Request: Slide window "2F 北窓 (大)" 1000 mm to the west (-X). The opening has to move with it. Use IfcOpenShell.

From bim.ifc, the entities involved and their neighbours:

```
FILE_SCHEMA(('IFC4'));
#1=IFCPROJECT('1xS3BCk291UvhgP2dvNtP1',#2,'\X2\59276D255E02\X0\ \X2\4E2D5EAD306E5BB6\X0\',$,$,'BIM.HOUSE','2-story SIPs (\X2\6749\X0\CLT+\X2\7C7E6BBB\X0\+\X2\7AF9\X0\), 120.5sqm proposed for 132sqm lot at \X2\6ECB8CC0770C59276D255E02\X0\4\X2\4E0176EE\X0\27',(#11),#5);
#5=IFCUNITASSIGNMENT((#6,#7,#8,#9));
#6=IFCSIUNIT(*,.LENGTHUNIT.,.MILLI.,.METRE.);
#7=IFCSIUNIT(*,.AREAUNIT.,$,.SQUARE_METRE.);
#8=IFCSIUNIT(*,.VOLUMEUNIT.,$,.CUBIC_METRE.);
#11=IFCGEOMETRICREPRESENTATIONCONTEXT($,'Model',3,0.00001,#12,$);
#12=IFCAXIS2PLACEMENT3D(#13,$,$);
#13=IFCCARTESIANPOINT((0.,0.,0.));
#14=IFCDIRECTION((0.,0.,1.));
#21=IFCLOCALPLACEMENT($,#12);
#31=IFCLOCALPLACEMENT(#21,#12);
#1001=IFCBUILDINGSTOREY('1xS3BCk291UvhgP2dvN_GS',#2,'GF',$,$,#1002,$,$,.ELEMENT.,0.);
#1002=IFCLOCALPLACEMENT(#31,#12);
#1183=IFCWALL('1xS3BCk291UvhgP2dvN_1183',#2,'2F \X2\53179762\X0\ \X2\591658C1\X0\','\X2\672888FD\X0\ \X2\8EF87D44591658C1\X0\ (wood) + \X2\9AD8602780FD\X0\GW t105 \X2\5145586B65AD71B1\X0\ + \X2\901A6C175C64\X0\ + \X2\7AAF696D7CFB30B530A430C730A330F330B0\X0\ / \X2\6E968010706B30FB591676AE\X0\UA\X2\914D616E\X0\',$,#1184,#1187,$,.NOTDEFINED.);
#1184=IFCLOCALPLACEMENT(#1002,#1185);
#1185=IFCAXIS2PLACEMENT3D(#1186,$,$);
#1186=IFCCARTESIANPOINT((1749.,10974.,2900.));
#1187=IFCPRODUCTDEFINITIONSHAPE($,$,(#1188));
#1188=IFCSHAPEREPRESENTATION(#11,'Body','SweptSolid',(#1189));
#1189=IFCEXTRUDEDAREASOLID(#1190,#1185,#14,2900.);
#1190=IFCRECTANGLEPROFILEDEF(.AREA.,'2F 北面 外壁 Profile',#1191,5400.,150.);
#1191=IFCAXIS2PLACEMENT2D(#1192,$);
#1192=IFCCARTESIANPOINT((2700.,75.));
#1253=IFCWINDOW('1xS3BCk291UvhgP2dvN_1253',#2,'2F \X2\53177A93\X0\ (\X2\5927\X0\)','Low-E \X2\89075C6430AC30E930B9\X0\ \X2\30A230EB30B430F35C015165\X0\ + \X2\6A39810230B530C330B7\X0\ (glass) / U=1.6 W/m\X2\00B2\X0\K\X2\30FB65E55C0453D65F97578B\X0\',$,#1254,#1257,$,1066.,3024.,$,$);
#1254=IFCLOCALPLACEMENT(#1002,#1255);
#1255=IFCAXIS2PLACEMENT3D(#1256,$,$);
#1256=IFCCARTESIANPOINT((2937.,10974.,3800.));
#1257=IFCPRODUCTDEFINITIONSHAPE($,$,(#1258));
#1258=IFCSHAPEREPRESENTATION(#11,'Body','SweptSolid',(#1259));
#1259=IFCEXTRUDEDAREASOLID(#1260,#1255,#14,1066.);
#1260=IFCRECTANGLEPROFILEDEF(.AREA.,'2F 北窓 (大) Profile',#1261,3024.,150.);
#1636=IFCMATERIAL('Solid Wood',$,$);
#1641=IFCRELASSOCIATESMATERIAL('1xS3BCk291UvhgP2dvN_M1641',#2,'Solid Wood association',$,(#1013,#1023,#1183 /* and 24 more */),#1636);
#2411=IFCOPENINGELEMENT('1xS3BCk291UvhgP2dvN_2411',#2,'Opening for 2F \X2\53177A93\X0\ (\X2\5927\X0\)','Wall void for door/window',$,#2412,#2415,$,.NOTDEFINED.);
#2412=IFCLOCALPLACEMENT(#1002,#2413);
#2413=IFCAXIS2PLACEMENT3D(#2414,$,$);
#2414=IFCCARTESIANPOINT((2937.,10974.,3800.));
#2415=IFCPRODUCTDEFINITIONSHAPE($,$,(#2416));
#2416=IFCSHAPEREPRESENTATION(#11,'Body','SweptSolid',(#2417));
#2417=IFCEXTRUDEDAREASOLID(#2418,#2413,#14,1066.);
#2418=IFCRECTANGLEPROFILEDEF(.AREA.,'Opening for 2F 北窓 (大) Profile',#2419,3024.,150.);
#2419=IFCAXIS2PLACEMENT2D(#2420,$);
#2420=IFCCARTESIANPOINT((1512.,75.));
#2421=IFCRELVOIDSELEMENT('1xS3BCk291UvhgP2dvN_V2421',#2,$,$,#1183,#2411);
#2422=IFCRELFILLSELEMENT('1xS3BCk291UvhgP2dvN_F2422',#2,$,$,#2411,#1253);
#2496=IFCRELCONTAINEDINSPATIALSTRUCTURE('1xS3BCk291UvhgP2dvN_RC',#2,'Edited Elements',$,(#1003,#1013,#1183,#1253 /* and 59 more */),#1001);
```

```python
import ifcopenshell
import ifcopenshell.api.geometry
import ifcopenshell.util.placement

model = ifcopenshell.open("bim.ifc")

window = model.by_guid("1xS3BCk291UvhgP2dvN_1253")
opening = window.FillsVoids[0].RelatingOpeningElement
wall = opening.VoidsElements[0].RelatingBuildingElement

wall_matrix = ifcopenshell.util.placement.get_local_placement(wall.ObjectPlacement)
shift = wall_matrix[:3, 0] * -1000.0
before = ifcopenshell.util.placement.get_local_placement(window.ObjectPlacement)[:3, 3].copy()

# The window is not placed relative to its opening, so move both.
for product in (opening, window):
    matrix = ifcopenshell.util.placement.get_local_placement(product.ObjectPlacement)
    matrix[:3, 3] += shift
    ifcopenshell.api.geometry.edit_object_placement(model, product=product, matrix=matrix, is_si=False)

after = ifcopenshell.util.placement.get_local_placement(window.ObjectPlacement)[:3, 3]
print("window moved by", (after - before).round(3) + 0.0)

model.write("bim_updated.ifc")
```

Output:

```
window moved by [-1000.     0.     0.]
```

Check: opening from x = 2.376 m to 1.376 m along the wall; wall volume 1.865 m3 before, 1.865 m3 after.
